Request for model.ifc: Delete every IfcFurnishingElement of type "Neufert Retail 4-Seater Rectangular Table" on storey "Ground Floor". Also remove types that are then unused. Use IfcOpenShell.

First a look at what the model holds.

```python
import ifcopenshell
import ifcopenshell.util.element

model = ifcopenshell.open("model.ifc")
print(model.schema)
storey = next(s for s in model.by_type("IfcBuildingStorey") if s.Name == "Ground Floor")
furniture = [e for e in ifcopenshell.util.element.get_decomposition(storey) if e.is_a("IfcFurnishingElement")]
seen = {}
for e in furniture:
    element_type = ifcopenshell.util.element.get_type(e)
    name = element_type.Name if element_type not in (None, e) else None
    seen[name] = seen.get(name, 0) + 1
for name, count in sorted(seen.items(), key=str):
    print(count, "x", name)
```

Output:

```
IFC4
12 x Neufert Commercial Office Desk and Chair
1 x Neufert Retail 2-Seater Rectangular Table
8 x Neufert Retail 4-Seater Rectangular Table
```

```python
import ifcopenshell
import ifcopenshell.api.root
import ifcopenshell.util.element

model = ifcopenshell.open("model.ifc")

storey = next(s for s in model.by_type("IfcBuildingStorey") if s.Name == "Ground Floor")
furniture = [e for e in ifcopenshell.util.element.get_decomposition(storey) if e.is_a("IfcFurnishingElement")]
targets = [e for e in furniture if (t := ifcopenshell.util.element.get_type(e)) not in (None, e) and t.Name == "Neufert Retail 4-Seater Rectangular Table"]
types = {ifcopenshell.util.element.get_type(e) for e in targets} - {None, *targets}

for e in targets:
    ifcopenshell.api.root.remove_product(model, product=e)
print(len(targets), "removed")

unused = [t for t in types if not ifcopenshell.util.element.get_types(t)]
for t in unused:
    ifcopenshell.api.root.remove_product(model, product=t)
print(len(unused), "unused types removed")

model.write("model_updated.ifc")
```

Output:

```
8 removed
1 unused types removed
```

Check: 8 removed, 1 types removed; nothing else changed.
